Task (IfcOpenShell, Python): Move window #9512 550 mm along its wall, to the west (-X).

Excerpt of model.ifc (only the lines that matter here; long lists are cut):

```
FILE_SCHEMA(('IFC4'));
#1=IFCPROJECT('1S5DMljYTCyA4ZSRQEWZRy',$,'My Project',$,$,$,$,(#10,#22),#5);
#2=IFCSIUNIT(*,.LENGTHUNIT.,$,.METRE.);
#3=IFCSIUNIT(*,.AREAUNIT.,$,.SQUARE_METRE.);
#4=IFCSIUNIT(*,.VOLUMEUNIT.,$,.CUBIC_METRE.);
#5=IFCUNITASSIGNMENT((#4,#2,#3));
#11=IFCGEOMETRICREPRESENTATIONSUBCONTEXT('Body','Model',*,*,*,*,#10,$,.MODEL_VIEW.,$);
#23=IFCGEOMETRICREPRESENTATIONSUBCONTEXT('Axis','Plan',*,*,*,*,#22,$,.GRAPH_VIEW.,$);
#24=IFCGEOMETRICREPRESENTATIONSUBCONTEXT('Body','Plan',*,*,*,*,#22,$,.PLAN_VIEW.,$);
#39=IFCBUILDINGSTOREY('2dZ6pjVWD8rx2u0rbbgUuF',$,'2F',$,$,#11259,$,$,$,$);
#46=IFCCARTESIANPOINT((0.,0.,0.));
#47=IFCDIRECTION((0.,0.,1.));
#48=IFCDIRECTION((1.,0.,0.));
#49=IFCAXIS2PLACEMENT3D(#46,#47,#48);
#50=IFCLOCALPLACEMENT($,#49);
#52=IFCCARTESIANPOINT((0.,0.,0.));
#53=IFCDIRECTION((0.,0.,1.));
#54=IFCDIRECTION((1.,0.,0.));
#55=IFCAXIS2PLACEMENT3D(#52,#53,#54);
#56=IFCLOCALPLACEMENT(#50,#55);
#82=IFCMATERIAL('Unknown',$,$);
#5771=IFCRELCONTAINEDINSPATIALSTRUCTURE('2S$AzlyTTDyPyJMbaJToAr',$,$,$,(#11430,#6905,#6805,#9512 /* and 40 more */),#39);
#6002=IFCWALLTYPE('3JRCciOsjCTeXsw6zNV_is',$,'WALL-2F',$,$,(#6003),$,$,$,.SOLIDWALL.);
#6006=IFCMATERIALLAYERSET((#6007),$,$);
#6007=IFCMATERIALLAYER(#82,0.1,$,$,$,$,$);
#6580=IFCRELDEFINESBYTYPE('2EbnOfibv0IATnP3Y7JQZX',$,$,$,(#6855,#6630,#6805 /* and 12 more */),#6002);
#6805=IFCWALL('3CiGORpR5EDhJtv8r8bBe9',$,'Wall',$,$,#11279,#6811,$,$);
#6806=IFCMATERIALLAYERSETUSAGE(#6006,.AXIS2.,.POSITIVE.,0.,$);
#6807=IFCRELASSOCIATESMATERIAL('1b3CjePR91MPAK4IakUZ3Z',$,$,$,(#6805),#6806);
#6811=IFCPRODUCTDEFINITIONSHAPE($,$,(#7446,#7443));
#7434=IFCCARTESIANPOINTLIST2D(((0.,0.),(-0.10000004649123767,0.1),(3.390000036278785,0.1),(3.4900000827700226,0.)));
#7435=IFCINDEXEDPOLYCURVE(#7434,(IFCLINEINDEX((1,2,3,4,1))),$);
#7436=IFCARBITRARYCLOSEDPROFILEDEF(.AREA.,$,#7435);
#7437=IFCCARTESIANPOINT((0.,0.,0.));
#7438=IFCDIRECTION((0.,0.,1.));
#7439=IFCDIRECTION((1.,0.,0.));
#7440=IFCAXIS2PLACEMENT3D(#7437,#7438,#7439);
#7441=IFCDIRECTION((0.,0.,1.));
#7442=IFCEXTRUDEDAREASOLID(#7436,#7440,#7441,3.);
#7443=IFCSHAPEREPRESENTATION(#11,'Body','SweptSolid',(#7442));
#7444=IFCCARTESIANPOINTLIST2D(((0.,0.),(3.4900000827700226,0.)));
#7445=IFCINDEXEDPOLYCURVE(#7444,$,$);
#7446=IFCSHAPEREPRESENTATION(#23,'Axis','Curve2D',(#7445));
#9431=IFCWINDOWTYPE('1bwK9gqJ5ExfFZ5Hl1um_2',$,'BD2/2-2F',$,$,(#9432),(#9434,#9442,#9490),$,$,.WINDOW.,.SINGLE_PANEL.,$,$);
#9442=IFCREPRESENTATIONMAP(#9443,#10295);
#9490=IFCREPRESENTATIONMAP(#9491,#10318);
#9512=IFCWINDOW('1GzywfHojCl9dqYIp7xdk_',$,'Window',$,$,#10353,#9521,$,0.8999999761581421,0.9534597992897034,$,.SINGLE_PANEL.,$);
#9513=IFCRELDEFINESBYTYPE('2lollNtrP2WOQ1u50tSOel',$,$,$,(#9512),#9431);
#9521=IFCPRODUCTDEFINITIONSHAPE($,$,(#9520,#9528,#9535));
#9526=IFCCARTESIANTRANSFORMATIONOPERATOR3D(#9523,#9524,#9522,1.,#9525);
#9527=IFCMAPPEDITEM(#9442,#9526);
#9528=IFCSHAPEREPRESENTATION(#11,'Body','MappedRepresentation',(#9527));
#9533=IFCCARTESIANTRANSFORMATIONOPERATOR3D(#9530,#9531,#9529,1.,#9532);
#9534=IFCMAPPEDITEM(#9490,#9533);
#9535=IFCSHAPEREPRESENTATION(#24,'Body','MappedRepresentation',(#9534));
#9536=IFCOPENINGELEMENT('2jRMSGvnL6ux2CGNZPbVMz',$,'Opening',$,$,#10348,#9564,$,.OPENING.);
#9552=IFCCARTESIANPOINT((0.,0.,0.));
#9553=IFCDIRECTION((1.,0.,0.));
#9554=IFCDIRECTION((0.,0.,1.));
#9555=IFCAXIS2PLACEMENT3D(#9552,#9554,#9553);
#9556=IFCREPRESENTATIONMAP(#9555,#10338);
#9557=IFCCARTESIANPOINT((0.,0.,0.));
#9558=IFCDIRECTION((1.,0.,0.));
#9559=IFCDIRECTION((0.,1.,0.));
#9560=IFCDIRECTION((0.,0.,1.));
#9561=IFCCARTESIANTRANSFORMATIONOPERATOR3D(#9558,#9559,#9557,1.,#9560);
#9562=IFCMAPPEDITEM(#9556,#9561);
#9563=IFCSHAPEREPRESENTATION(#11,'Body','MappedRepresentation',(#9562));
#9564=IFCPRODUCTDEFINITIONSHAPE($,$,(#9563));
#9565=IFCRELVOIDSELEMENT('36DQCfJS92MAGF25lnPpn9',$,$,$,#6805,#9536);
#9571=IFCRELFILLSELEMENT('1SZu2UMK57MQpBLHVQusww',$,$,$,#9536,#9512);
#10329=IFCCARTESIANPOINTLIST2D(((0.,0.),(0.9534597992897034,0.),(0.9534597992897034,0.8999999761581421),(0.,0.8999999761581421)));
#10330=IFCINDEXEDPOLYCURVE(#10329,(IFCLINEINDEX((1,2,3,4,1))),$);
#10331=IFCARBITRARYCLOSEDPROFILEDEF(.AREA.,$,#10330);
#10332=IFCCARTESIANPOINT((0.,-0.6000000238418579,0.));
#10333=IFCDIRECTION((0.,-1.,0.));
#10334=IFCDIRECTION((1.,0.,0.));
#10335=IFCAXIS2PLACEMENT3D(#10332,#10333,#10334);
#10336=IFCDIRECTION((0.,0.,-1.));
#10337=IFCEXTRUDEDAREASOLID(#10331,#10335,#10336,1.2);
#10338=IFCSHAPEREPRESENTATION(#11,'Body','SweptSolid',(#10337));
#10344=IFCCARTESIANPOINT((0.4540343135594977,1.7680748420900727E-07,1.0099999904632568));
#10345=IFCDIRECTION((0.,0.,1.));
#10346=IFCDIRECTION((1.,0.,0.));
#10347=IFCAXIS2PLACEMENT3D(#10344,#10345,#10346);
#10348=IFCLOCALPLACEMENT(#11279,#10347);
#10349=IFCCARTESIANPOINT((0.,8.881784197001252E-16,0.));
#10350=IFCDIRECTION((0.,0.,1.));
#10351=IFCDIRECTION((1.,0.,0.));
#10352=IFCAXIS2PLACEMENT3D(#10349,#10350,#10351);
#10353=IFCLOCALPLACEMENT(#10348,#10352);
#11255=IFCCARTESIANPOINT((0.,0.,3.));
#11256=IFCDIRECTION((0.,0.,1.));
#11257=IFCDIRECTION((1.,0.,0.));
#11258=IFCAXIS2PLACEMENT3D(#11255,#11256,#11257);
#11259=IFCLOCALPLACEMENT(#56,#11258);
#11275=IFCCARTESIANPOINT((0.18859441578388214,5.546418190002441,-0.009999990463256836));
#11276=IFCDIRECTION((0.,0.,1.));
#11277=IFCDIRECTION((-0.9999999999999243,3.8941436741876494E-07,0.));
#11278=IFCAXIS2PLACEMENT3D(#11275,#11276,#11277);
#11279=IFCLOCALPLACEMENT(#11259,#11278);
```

```python
import ifcopenshell
import ifcopenshell.api.geometry
import ifcopenshell.util.placement
import ifcopenshell.util.unit

model = ifcopenshell.open("model.ifc")
unit_scale = ifcopenshell.util.unit.calculate_unit_scale(model)

window = model.by_guid("1GzywfHojCl9dqYIp7xdk_")
opening = window.FillsVoids[0].RelatingOpeningElement
wall = opening.VoidsElements[0].RelatingBuildingElement

wall_matrix = ifcopenshell.util.placement.get_local_placement(wall.ObjectPlacement)
shift = wall_matrix[:3, 0] * 0.55 / unit_scale
before = ifcopenshell.util.placement.get_local_placement(window.ObjectPlacement)[:3, 3].copy()

# The window is placed relative to its opening, so it follows when the opening moves.
matrix = ifcopenshell.util.placement.get_local_placement(opening.ObjectPlacement)
matrix[:3, 3] += shift
ifcopenshell.api.geometry.edit_object_placement(
    model, product=opening, matrix=matrix, is_si=False, should_transform_children=True
)

after = ifcopenshell.util.placement.get_local_placement(window.ObjectPlacement)[:3, 3]
print("window moved by", (after - before).round(3) + 0.0)

model.write("model_edited.ifc")
```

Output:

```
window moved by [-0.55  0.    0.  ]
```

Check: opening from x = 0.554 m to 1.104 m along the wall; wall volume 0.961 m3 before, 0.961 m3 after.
